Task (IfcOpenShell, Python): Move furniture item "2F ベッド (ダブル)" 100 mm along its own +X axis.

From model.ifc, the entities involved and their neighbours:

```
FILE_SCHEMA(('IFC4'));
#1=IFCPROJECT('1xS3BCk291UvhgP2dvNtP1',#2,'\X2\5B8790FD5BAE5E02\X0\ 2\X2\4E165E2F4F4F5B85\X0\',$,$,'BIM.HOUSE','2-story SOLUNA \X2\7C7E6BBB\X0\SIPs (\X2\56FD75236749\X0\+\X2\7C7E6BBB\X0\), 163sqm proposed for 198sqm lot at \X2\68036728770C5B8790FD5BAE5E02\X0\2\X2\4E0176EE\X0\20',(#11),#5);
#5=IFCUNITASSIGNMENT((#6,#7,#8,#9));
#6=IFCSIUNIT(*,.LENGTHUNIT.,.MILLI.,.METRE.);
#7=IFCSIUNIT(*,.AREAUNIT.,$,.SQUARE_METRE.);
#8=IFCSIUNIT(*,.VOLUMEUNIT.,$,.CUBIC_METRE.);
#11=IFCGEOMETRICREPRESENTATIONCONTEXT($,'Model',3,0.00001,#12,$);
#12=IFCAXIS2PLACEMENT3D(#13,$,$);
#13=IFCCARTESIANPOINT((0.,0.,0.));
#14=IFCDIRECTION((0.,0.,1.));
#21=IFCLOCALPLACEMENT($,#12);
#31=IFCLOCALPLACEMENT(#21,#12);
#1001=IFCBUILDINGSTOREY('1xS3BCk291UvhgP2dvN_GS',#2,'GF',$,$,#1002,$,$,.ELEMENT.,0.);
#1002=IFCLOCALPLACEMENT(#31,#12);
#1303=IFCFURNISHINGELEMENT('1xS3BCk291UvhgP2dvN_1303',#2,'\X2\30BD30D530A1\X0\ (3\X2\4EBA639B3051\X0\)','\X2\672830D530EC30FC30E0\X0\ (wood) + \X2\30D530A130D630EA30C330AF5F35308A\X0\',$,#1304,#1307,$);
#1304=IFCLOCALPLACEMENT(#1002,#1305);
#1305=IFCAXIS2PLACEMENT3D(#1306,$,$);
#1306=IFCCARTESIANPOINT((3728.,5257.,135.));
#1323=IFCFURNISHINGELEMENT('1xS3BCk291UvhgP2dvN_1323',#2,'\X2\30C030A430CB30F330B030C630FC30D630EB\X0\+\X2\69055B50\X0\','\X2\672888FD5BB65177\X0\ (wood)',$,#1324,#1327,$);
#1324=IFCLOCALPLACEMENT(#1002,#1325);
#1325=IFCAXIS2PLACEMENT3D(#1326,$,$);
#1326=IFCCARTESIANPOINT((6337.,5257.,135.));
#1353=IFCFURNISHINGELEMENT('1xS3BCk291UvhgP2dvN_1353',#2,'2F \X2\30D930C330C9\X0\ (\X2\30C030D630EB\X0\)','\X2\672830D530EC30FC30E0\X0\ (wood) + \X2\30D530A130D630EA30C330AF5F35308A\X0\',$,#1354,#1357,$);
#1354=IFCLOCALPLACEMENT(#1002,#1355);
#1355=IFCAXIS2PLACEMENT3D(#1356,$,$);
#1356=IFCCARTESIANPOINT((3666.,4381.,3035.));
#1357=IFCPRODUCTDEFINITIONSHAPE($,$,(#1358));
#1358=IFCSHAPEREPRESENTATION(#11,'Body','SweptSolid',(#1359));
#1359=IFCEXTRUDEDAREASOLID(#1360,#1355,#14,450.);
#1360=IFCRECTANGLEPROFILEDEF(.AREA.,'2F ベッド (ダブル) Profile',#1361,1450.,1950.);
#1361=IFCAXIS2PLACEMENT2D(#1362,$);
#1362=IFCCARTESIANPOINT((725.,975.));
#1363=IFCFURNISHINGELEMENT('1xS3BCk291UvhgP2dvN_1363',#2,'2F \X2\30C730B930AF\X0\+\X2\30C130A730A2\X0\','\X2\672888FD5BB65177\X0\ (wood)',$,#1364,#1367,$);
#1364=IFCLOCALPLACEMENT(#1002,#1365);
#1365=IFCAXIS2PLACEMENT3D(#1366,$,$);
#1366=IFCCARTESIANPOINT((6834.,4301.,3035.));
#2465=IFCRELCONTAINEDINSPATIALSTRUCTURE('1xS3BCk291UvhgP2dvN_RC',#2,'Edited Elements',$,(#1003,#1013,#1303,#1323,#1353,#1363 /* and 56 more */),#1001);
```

```python
import ifcopenshell
import ifcopenshell.api.geometry
import ifcopenshell.util.placement

model = ifcopenshell.open("model.ifc")

item = model.by_guid("1xS3BCk291UvhgP2dvN_1353")
matrix = ifcopenshell.util.placement.get_local_placement(item.ObjectPlacement)
matrix[:3, 3] += matrix[:3, 0] * 100.0
ifcopenshell.api.geometry.edit_object_placement(model, product=item, matrix=matrix, is_si=False)

print(ifcopenshell.util.placement.get_local_placement(item.ObjectPlacement).round(3) + 0.0)

model.write("model_v2.ifc")
```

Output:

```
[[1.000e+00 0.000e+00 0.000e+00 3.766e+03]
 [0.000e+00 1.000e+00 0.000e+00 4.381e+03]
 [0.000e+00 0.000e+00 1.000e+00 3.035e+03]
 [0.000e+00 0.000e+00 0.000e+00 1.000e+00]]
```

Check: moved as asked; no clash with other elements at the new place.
